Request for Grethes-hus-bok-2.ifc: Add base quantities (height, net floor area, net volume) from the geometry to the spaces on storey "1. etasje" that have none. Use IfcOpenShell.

First a look at what the model holds.

```python
import ifcopenshell
import ifcopenshell.util.element
import ifcopenshell.util.unit

model = ifcopenshell.open("Grethes-hus-bok-2.ifc")
print(model.schema)
for unit_type in ("LENGTHUNIT", "AREAUNIT", "VOLUMEUNIT"):
    print(unit_type, ifcopenshell.util.unit.calculate_unit_scale(model, unit_type))
storey = next(s for s in model.by_type("IfcBuildingStorey") if s.Name == "1. etasje")
spaces = [e for e in ifcopenshell.util.element.get_decomposition(storey) if e.is_a("IfcSpace")]
for e in sorted(spaces, key=lambda e: e.id()):
    print(e.id(), e.is_a(), e.Name, list(ifcopenshell.util.element.get_psets(e, qtos_only=True)), sep=" | ")
```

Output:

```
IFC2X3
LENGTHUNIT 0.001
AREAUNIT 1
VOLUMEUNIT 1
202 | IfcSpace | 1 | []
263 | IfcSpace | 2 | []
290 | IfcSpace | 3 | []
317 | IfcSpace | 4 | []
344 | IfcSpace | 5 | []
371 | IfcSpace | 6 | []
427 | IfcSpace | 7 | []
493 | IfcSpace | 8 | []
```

```python
import ifcopenshell
import ifcopenshell.api.pset
import ifcopenshell.geom
import ifcopenshell.util.element
import ifcopenshell.util.shape
import ifcopenshell.util.unit

model = ifcopenshell.open("Grethes-hus-bok-2.ifc")
unit_scale = ifcopenshell.util.unit.calculate_unit_scale(model)
area_scale = ifcopenshell.util.unit.calculate_unit_scale(model, "AREAUNIT")
volume_scale = ifcopenshell.util.unit.calculate_unit_scale(model, "VOLUMEUNIT")
settings = ifcopenshell.geom.settings()

storey = next(s for s in model.by_type("IfcBuildingStorey") if s.Name == "1. etasje")
spaces = [e for e in ifcopenshell.util.element.get_decomposition(storey) if e.is_a("IfcSpace")]

for e in sorted(spaces, key=lambda e: e.id()):
    if ifcopenshell.util.element.get_psets(e, qtos_only=True, should_inherit=False):
        continue
    # Geometry comes back in metres, in the element's own axes.
    shape = ifcopenshell.geom.create_shape(settings, e)
    values = {
        "Height": ifcopenshell.util.shape.get_z(shape.geometry) / unit_scale,
        "NetFloorArea": ifcopenshell.util.shape.get_footprint_area(shape.geometry) / area_scale,
        "NetVolume": ifcopenshell.util.shape.get_volume(shape.geometry) / volume_scale,
    }
    qto = ifcopenshell.api.pset.add_qto(model, product=e, name="BaseQuantities")
    ifcopenshell.api.pset.edit_qto(model, qto=qto, properties=values)
    print(e.id(), {k: round(v, 3) for k, v in values.items()})

model.write("Grethes-hus-bok-2_updated.ifc")
```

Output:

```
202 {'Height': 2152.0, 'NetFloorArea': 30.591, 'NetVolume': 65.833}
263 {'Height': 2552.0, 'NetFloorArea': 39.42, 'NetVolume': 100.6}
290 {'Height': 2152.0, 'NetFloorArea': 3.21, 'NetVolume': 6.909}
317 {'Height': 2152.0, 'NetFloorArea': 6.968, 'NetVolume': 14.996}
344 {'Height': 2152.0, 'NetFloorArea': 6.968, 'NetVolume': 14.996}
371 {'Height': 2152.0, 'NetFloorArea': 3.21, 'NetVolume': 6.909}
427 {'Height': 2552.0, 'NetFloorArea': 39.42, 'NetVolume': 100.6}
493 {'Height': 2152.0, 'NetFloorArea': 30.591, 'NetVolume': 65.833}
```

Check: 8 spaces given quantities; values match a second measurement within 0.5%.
